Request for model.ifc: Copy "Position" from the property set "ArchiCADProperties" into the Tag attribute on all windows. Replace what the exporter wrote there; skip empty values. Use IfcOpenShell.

First a look at what the model holds.

```python
import ifcopenshell
import ifcopenshell.util.element

model = ifcopenshell.open("model.ifc")
print(model.schema)
windows = model.by_type("IfcWindow")
print(len(windows), "windows")
for e in windows[:8]:
    source = ifcopenshell.util.element.get_pset(e, "ArchiCADProperties", "Position")
    target = e.Tag
    print(e.id(), repr(source), repr(target), sep=" | ")
```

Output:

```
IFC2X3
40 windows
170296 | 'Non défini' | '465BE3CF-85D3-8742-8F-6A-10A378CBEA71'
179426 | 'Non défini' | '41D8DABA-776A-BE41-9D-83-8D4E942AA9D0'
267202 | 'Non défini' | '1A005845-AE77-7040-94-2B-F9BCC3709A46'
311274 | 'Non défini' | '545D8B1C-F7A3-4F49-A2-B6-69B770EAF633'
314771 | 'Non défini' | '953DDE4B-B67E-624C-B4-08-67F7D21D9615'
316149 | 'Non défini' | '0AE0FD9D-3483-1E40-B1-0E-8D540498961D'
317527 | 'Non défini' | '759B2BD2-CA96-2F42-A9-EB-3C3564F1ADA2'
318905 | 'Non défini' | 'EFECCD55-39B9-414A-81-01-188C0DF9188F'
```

```python
import ifcopenshell
import ifcopenshell.util.element

model = ifcopenshell.open("model.ifc")

count = 0
for e in model.by_type("IfcWindow"):
    value = ifcopenshell.util.element.get_pset(e, "ArchiCADProperties", "Position")
    current = e.Tag
    if not value or not value.strip() or current == value:
        continue
    e.Tag = value
    count += 1

print(count, "windows updated")

model.write("model_edited.ifc")
```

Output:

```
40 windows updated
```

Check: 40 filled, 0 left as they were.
